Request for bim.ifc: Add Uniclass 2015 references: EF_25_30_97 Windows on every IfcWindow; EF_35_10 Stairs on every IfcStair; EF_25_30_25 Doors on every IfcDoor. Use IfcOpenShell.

First a look at what the model holds.

```python
import ifcopenshell

model = ifcopenshell.open("bim.ifc")
print(model.schema)
print("classifications:", [c.Name for c in model.by_type("IfcClassification")])
for ifc_class in ("IfcDoor", "IfcRoof", "IfcStair", "IfcWall", "IfcWindow"):
    print(ifc_class, len(model.by_type(ifc_class)))
```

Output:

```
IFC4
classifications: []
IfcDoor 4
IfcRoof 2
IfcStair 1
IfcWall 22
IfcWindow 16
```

```python
import ifcopenshell
import ifcopenshell.api.classification

model = ifcopenshell.open("bim.ifc")

system = ifcopenshell.api.classification.add_classification(model, classification="Uniclass 2015")

codes = {
    "IfcWindow": ("EF_25_30_97", "Windows"),
    "IfcStair": ("EF_35_10", "Stairs"),
    "IfcDoor": ("EF_25_30_25", "Doors"),
}
for ifc_class, (code, name) in codes.items():
    products = model.by_type(ifc_class)
    ifcopenshell.api.classification.add_reference(
        model, products=products, classification=system, identification=code, name=name
    )
    print(code, len(products))

model.write("bim_v2.ifc")
```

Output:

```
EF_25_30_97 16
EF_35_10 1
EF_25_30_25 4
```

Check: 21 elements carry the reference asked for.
